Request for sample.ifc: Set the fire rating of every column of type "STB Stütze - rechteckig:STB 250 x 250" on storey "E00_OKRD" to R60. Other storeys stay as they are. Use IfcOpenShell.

First a look at what the model holds.

```python
import ifcopenshell
import ifcopenshell.util.element

model = ifcopenshell.open("sample.ifc")
print(model.schema)
storey = next(s for s in model.by_type("IfcBuildingStorey") if s.Name == "E00_OKRD")
columns = [e for e in ifcopenshell.util.element.get_decomposition(storey) if e.is_a("IfcColumn")]
seen = {}
for e in columns:
    element_type = ifcopenshell.util.element.get_type(e)
    key = (element_type.Name if element_type != e and element_type else None, ifcopenshell.util.element.get_pset(e, "Pset_ColumnCommon", "FireRating"))
    seen[key] = seen.get(key, 0) + 1
for (name, value), count in sorted(seen.items(), key=str):
    print(count, "x", name, "|", value)
```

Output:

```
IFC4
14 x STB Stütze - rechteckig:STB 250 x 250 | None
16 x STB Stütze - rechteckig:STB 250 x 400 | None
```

```python
import ifcopenshell
import ifcopenshell.api.pset
import ifcopenshell.util.element

model = ifcopenshell.open("sample.ifc")

storey = next(s for s in model.by_type("IfcBuildingStorey") if s.Name == "E00_OKRD")
columns = [e for e in ifcopenshell.util.element.get_decomposition(storey) if e.is_a("IfcColumn")]

count = 0
for e in columns:
    element_type = ifcopenshell.util.element.get_type(e)
    if element_type in (None, e) or element_type.Name != "STB Stütze - rechteckig:STB 250 x 250":
        continue
    # add_pset returns the element's existing set when there is one.
    pset = ifcopenshell.api.pset.add_pset(model, product=e, name="Pset_ColumnCommon")
    ifcopenshell.api.pset.edit_pset(model, pset=pset, properties={"FireRating": "R60"})
    count += 1

print(count, "columns updated")

model.write("sample_rev.ifc")
```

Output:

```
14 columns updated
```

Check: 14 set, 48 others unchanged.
